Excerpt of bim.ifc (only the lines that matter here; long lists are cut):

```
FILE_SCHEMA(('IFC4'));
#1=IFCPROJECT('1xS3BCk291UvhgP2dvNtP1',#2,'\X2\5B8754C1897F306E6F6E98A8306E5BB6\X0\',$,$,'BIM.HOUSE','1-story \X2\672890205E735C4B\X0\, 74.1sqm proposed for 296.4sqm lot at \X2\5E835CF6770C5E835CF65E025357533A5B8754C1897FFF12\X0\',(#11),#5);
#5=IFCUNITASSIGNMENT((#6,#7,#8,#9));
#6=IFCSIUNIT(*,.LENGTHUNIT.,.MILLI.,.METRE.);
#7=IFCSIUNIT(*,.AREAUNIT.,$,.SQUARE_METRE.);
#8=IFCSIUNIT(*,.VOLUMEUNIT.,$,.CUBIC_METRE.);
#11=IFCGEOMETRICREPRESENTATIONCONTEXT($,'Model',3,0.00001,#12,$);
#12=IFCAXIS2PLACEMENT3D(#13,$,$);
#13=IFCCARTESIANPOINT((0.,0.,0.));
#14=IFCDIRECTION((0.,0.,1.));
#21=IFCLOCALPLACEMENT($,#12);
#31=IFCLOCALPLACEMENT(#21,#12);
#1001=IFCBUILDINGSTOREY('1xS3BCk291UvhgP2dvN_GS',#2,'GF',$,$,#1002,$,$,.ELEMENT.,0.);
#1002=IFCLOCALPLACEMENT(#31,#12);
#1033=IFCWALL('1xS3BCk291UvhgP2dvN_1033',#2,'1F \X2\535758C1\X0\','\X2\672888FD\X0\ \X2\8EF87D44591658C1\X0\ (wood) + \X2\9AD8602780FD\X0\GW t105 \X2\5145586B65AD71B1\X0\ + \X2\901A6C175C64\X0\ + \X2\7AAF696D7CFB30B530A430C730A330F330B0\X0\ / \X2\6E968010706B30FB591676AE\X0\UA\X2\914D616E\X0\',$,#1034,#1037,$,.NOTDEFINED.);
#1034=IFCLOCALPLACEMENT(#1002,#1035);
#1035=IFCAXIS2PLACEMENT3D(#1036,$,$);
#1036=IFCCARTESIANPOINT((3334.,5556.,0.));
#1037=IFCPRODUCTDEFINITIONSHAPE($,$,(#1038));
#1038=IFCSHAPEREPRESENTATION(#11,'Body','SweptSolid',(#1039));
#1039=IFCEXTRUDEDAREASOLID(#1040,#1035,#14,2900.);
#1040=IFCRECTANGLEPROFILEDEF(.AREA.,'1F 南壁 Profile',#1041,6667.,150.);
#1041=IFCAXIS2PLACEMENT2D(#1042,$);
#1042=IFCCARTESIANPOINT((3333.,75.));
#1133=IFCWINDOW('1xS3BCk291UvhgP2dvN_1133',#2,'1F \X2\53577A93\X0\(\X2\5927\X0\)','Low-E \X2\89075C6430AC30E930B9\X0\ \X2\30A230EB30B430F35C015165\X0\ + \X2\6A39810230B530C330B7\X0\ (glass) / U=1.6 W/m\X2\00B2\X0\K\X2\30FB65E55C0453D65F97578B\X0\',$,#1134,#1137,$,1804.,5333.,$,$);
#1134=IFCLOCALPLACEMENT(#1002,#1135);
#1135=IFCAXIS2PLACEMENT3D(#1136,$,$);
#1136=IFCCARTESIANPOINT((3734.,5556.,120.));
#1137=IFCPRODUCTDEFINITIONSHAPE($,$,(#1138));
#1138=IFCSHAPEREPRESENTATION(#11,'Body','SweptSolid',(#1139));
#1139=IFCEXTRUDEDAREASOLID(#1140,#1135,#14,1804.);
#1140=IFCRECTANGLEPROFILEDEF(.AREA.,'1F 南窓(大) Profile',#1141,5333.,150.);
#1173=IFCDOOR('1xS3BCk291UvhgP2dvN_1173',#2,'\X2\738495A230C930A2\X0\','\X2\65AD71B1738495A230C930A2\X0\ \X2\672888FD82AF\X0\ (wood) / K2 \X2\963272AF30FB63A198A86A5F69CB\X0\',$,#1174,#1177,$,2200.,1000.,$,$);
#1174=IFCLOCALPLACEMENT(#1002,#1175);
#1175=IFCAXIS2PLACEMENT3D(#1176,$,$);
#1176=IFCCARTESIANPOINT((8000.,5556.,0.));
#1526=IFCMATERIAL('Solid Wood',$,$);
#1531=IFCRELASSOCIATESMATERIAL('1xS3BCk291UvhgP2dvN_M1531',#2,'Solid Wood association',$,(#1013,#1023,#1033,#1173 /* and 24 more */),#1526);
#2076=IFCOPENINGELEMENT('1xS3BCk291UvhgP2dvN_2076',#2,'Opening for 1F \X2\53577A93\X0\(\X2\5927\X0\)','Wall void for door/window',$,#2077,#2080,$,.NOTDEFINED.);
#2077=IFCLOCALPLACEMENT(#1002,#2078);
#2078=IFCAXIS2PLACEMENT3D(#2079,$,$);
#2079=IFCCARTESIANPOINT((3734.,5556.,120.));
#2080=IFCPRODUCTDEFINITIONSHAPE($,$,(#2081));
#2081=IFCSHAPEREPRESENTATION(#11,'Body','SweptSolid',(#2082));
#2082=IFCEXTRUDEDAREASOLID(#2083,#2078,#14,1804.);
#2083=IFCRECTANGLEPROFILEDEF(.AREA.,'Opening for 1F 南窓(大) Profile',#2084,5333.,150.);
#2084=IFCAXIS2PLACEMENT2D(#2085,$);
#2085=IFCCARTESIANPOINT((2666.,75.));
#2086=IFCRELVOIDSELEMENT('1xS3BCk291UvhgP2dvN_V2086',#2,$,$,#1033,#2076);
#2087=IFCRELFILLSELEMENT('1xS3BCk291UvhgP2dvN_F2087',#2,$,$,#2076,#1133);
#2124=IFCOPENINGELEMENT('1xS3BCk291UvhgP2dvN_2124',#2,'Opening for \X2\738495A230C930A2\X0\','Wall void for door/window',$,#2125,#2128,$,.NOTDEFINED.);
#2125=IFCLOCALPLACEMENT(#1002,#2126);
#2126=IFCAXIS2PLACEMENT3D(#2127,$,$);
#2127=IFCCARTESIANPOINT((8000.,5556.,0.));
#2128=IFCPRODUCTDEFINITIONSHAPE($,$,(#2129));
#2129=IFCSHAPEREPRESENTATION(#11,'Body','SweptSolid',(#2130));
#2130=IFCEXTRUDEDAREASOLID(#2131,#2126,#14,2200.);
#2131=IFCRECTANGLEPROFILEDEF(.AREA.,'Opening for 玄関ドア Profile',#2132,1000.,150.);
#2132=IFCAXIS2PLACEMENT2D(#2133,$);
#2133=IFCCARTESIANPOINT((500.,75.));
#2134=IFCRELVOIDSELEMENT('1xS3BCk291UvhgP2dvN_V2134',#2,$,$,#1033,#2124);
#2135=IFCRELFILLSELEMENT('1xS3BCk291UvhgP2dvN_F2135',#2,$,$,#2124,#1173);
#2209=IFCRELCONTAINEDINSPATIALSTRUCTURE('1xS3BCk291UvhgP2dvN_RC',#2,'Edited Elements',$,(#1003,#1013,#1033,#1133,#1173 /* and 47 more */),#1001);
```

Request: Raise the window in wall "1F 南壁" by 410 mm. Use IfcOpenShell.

```python
import numpy as np
import ifcopenshell
import ifcopenshell.api.geometry
import ifcopenshell.util.placement
import ifcopenshell.util.unit

model = ifcopenshell.open("bim.ifc")
unit_scale = ifcopenshell.util.unit.calculate_unit_scale(model)

window = model.by_guid("1xS3BCk291UvhgP2dvN_1133")
opening = window.FillsVoids[0].RelatingOpeningElement
dz = 0.41 / unit_scale

shift = np.array([0.0, 0.0, dz])
# The window is not placed relative to its opening, so move both.
for product in (opening, window):
    matrix = ifcopenshell.util.placement.get_local_placement(product.ObjectPlacement)
    matrix[:3, 3] += shift
    ifcopenshell.api.geometry.edit_object_placement(model, product=product, matrix=matrix, is_si=False)

print(f"moved by {dz * unit_scale:+.3f} m")

model.write("bim_updated.ifc")
```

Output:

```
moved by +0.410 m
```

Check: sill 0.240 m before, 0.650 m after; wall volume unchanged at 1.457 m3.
